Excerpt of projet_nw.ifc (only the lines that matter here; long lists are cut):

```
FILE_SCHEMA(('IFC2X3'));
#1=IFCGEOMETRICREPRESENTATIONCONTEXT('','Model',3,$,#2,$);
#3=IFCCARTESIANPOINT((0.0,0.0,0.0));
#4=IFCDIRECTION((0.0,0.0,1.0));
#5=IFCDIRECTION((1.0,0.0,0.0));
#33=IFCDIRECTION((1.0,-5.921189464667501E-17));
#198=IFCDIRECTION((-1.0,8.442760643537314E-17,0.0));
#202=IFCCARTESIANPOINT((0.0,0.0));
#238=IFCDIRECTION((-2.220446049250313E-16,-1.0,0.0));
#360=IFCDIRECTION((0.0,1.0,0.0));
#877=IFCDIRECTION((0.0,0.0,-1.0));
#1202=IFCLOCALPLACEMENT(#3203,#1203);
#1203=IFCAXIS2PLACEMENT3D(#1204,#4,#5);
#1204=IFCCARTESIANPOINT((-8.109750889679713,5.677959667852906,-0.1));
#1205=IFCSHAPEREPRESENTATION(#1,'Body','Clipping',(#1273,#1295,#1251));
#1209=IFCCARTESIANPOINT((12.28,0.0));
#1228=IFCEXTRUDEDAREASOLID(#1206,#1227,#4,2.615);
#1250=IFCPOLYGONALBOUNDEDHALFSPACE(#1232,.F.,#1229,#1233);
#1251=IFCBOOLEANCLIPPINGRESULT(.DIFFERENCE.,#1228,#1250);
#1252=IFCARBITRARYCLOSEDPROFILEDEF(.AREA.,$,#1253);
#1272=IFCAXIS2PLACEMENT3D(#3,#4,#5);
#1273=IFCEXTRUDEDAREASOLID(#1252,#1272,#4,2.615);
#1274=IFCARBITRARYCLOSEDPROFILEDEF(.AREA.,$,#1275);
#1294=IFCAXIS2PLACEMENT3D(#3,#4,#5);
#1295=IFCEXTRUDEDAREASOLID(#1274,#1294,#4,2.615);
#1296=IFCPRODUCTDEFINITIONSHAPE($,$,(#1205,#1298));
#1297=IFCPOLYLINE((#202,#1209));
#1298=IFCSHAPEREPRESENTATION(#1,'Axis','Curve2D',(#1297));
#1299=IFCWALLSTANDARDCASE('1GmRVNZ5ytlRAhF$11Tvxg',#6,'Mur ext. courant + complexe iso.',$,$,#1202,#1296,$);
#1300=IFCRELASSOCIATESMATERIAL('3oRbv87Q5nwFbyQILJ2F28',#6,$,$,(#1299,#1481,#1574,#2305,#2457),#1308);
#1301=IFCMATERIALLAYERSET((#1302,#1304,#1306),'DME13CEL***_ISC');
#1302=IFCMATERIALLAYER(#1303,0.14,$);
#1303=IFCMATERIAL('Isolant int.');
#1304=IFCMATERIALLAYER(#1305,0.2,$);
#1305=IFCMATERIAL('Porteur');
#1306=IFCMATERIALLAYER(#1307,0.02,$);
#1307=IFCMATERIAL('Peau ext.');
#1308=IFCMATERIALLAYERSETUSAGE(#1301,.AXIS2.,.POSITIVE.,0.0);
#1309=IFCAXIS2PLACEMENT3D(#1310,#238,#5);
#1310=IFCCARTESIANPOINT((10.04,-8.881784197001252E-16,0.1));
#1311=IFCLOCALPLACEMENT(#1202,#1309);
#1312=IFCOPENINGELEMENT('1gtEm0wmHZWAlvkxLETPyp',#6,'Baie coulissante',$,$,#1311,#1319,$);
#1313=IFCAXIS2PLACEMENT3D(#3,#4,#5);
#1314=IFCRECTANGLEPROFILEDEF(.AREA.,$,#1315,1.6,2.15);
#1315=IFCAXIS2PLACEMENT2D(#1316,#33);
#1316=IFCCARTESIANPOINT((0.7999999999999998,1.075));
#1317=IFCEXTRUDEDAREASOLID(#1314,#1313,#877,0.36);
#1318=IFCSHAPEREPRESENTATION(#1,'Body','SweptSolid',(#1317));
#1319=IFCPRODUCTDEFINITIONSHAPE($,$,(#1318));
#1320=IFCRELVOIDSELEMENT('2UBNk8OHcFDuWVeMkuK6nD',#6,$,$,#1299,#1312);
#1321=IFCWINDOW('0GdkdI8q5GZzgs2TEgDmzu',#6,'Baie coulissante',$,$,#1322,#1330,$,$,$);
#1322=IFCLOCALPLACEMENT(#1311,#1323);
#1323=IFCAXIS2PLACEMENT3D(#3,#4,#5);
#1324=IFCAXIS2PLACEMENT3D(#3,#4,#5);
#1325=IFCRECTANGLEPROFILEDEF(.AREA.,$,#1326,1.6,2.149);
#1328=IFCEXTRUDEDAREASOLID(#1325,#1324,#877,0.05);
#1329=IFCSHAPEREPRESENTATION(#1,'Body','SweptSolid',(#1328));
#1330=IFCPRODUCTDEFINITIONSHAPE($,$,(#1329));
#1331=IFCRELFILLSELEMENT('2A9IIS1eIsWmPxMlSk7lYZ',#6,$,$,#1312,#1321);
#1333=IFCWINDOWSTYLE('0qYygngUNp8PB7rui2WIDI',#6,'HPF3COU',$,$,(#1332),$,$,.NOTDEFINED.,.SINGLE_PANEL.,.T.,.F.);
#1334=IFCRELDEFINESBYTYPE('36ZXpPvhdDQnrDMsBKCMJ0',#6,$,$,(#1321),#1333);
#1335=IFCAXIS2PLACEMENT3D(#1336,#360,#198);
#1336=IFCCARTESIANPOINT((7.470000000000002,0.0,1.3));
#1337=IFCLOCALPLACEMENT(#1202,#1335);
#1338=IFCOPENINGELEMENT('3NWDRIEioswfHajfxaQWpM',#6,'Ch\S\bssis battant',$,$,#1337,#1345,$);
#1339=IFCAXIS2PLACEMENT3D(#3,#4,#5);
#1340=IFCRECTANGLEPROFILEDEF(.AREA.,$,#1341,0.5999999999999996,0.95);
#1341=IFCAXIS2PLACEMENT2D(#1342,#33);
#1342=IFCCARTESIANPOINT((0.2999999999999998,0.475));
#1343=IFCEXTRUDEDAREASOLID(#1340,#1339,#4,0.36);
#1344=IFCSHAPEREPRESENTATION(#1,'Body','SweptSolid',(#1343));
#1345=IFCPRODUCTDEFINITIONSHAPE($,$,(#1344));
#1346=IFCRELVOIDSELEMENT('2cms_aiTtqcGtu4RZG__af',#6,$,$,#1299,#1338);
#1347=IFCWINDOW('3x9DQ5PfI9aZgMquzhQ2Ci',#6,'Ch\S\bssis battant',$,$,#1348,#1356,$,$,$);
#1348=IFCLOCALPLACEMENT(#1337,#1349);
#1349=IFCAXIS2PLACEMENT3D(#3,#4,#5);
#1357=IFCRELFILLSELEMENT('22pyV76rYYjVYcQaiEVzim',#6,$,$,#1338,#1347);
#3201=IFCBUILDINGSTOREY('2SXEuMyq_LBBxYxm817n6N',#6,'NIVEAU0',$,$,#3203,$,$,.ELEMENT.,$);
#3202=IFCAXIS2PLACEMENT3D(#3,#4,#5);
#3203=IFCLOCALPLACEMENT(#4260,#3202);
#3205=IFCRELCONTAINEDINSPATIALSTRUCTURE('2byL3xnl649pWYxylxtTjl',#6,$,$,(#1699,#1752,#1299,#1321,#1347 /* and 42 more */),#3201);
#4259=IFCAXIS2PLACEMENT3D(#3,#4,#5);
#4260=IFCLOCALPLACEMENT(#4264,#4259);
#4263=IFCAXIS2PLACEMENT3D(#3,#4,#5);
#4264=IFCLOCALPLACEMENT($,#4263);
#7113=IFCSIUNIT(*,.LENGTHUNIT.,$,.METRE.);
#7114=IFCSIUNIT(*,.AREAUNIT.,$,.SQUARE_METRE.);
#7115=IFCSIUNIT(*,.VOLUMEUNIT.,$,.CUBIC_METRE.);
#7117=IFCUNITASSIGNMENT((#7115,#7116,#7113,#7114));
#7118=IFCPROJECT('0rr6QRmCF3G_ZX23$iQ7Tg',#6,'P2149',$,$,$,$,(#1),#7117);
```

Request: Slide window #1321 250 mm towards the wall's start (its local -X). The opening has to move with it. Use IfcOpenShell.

```python
import ifcopenshell
import ifcopenshell.api.geometry
import ifcopenshell.util.placement
import ifcopenshell.util.unit

model = ifcopenshell.open("projet_nw.ifc")
unit_scale = ifcopenshell.util.unit.calculate_unit_scale(model)

window = model.by_guid("0GdkdI8q5GZzgs2TEgDmzu")
opening = window.FillsVoids[0].RelatingOpeningElement
wall = opening.VoidsElements[0].RelatingBuildingElement

wall_matrix = ifcopenshell.util.placement.get_local_placement(wall.ObjectPlacement)
shift = wall_matrix[:3, 0] * -0.25 / unit_scale
before = ifcopenshell.util.placement.get_local_placement(window.ObjectPlacement)[:3, 3].copy()

# The window is placed relative to its opening, so it follows when the opening moves.
matrix = ifcopenshell.util.placement.get_local_placement(opening.ObjectPlacement)
matrix[:3, 3] += shift
ifcopenshell.api.geometry.edit_object_placement(
    model, product=opening, matrix=matrix, is_si=False, should_transform_children=True
)

after = ifcopenshell.util.placement.get_local_placement(window.ObjectPlacement)[:3, 3]
print("window moved by", (after - before).round(3) + 0.0)

model.write("projet_nw-out.ifc")
```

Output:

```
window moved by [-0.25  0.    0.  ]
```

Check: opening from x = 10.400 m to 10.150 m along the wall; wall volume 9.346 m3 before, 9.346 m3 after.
